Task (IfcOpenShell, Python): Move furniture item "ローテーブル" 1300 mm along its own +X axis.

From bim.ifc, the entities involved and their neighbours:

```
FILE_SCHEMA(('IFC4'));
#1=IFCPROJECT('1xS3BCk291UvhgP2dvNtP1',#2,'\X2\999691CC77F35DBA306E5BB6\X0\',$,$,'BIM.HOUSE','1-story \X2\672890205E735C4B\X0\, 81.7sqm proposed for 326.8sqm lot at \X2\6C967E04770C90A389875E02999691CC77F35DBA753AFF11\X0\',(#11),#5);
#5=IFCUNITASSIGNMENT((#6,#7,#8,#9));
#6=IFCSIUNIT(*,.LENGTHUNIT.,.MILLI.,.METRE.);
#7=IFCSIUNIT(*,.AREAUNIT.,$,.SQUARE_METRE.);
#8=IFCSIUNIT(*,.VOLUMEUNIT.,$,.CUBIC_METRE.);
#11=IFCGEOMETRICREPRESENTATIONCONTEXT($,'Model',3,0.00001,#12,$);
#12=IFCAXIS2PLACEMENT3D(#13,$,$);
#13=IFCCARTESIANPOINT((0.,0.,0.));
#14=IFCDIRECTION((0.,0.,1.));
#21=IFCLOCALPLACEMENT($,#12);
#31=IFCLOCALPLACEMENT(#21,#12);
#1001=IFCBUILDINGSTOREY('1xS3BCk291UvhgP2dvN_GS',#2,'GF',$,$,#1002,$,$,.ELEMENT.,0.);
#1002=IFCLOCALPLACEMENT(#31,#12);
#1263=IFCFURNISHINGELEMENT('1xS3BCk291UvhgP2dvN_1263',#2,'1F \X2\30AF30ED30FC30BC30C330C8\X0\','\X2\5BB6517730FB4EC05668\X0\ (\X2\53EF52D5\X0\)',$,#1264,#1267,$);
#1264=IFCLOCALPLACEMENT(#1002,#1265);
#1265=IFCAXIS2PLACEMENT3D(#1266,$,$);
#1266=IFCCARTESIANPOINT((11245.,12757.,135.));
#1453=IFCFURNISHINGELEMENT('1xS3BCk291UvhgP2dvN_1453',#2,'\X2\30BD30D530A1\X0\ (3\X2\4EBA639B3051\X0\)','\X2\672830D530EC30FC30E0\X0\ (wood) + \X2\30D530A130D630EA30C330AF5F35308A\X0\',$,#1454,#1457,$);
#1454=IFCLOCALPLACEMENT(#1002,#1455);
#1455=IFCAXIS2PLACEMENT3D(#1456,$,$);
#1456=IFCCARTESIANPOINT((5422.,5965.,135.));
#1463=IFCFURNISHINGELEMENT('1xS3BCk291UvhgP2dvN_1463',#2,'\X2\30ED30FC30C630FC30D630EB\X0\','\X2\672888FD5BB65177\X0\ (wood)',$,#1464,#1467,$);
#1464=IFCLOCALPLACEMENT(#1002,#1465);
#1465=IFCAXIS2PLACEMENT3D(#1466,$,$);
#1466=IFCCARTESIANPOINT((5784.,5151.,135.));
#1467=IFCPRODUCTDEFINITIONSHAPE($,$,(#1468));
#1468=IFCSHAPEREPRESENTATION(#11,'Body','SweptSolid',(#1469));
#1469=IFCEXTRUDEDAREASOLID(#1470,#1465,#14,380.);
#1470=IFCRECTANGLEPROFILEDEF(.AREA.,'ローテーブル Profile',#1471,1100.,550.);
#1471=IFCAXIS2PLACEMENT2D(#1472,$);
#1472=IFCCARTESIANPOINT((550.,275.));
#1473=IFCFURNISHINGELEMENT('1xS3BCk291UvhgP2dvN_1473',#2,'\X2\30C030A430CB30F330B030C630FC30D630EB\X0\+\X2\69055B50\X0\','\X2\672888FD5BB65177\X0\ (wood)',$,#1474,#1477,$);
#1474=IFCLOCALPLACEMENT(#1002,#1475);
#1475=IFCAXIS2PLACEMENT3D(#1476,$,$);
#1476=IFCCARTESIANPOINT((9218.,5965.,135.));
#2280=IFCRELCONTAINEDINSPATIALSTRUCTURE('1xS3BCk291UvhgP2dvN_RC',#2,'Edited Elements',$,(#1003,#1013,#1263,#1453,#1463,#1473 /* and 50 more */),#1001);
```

```python
import ifcopenshell
import ifcopenshell.api.geometry
import ifcopenshell.util.placement
import ifcopenshell.util.unit

model = ifcopenshell.open("bim.ifc")
unit_scale = ifcopenshell.util.unit.calculate_unit_scale(model)

item = model.by_id(1463)
matrix = ifcopenshell.util.placement.get_local_placement(item.ObjectPlacement)
matrix[:3, 3] += matrix[:3, 0] * 1.3 / unit_scale
ifcopenshell.api.geometry.edit_object_placement(model, product=item, matrix=matrix, is_si=False)

print(ifcopenshell.util.placement.get_local_placement(item.ObjectPlacement).round(3) + 0.0)

model.write("bim-out.ifc")
```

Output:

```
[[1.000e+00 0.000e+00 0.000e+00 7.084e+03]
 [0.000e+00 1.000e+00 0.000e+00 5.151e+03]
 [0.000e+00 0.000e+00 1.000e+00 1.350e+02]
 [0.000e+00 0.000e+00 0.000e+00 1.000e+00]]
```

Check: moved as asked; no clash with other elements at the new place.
